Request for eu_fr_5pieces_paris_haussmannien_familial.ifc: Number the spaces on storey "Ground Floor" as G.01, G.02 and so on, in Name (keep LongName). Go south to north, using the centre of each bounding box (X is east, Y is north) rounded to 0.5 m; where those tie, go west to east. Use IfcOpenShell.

First a look at what the model holds.

```python
import ifcopenshell
import ifcopenshell.util.element
import ifcopenshell.util.placement

model = ifcopenshell.open("eu_fr_5pieces_paris_haussmannien_familial.ifc")
print(model.schema)
storey = next(s for s in model.by_type("IfcBuildingStorey") if s.Name == "Ground Floor")
spaces = [e for e in ifcopenshell.util.element.get_decomposition(storey) if e.is_a("IfcSpace")]
for e in sorted(spaces, key=lambda e: e.id()):
    origin = ifcopenshell.util.placement.get_local_placement(e.ObjectPlacement)[:3, 3]
    print(e.id(), e.Name, e.LongName, origin.round(2) + 0.0, sep=" | ")
```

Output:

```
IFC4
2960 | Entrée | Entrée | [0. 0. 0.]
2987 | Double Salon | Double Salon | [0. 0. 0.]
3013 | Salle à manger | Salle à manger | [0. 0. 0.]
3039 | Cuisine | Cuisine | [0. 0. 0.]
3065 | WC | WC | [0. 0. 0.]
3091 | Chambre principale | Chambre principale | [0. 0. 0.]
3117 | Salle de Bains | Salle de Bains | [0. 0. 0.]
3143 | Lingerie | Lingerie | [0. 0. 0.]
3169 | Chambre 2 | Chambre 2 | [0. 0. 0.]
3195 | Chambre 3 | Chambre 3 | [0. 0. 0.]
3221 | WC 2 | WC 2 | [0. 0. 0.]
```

```python
import ifcopenshell
import ifcopenshell.geom
import ifcopenshell.util.element
import ifcopenshell.util.shape

model = ifcopenshell.open("eu_fr_5pieces_paris_haussmannien_familial.ifc")
settings = ifcopenshell.geom.settings()
settings.set("use-world-coords", True)


def centre(element):
    shape = ifcopenshell.geom.create_shape(settings, element)
    return ifcopenshell.util.shape.get_bbox_centroid(shape.geometry)


storey = next(s for s in model.by_type("IfcBuildingStorey") if s.Name == "Ground Floor")
spaces = [e for e in ifcopenshell.util.element.get_decomposition(storey) if e.is_a("IfcSpace")]

# Insertion points can sit at a corner or the storey origin, so sort by the geometry (in metres).
centres = {e: centre(e) for e in spaces}
spaces.sort(key=lambda e: (round(centres[e][1] / 0.5), centres[e][0]))

for i, e in enumerate(spaces, start=1):
    number = f"G.{i:02d}"
    e.Name = number
    print(e.id(), number)

model.write("eu_fr_5pieces_paris_haussmannien_familial_v2.ifc")
```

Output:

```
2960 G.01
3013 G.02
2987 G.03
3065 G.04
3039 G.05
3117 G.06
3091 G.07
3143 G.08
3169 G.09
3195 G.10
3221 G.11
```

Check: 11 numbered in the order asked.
